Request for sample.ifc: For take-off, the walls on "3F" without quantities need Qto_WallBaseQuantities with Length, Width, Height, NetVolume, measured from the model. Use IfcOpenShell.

First a look at what the model holds.

```python
import ifcopenshell
import ifcopenshell.util.element
import ifcopenshell.util.unit

model = ifcopenshell.open("sample.ifc")
print(model.schema)
for unit_type in ("LENGTHUNIT", "AREAUNIT", "VOLUMEUNIT"):
    print(unit_type, ifcopenshell.util.unit.calculate_unit_scale(model, unit_type))
storey = next(s for s in model.by_type("IfcBuildingStorey") if s.Name == "3F")
walls = [e for e in ifcopenshell.util.element.get_decomposition(storey) if e.is_a("IfcWall")]
for e in sorted(walls, key=lambda e: e.id()):
    print(e.id(), e.is_a(), e.Name, list(ifcopenshell.util.element.get_psets(e, qtos_only=True)), sep=" | ")
```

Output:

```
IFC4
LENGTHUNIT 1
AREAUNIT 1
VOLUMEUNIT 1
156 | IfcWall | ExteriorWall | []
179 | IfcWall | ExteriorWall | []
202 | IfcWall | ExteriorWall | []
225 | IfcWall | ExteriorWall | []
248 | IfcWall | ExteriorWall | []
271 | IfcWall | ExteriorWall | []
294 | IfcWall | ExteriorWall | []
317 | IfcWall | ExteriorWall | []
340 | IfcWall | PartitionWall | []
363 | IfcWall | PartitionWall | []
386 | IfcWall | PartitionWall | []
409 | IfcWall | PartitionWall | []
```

```python
import ifcopenshell
import ifcopenshell.api.pset
import ifcopenshell.geom
import ifcopenshell.util.element
import ifcopenshell.util.shape
import ifcopenshell.util.unit

model = ifcopenshell.open("sample.ifc")
unit_scale = ifcopenshell.util.unit.calculate_unit_scale(model)
volume_scale = ifcopenshell.util.unit.calculate_unit_scale(model, "VOLUMEUNIT")
settings = ifcopenshell.geom.settings()

storey = next(s for s in model.by_type("IfcBuildingStorey") if s.Name == "3F")
walls = [e for e in ifcopenshell.util.element.get_decomposition(storey) if e.is_a("IfcWall")]

for e in sorted(walls, key=lambda e: e.id()):
    if ifcopenshell.util.element.get_psets(e, qtos_only=True, should_inherit=False):
        continue
    # Geometry comes back in metres, in the element's own axes.
    shape = ifcopenshell.geom.create_shape(settings, e)
    values = {
        "Length": ifcopenshell.util.shape.get_x(shape.geometry) / unit_scale,
        "Width": ifcopenshell.util.shape.get_y(shape.geometry) / unit_scale,
        "Height": ifcopenshell.util.shape.get_z(shape.geometry) / unit_scale,
        "NetVolume": ifcopenshell.util.shape.get_volume(shape.geometry) / volume_scale,
    }
    qto = ifcopenshell.api.pset.add_qto(model, product=e, name="Qto_WallBaseQuantities")
    ifcopenshell.api.pset.edit_qto(model, qto=qto, properties=values)
    print(e.id(), {k: round(v, 3) for k, v in values.items()})

model.write("sample-out.ifc")
```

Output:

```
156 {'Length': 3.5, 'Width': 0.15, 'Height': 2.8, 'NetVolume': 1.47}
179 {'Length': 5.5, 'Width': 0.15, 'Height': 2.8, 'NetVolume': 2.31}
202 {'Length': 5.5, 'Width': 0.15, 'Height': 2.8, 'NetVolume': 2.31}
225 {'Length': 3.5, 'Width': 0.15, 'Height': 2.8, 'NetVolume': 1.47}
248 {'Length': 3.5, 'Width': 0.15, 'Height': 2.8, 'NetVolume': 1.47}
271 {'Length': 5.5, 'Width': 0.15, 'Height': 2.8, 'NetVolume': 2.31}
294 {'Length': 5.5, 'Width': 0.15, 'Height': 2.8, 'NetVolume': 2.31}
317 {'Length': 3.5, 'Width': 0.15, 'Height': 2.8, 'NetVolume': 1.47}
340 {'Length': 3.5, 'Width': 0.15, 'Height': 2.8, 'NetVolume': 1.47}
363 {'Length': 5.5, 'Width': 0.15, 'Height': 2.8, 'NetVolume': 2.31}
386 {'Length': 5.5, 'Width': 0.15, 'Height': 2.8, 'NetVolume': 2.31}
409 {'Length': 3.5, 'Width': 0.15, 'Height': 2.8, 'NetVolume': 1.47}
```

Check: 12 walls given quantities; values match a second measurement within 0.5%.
